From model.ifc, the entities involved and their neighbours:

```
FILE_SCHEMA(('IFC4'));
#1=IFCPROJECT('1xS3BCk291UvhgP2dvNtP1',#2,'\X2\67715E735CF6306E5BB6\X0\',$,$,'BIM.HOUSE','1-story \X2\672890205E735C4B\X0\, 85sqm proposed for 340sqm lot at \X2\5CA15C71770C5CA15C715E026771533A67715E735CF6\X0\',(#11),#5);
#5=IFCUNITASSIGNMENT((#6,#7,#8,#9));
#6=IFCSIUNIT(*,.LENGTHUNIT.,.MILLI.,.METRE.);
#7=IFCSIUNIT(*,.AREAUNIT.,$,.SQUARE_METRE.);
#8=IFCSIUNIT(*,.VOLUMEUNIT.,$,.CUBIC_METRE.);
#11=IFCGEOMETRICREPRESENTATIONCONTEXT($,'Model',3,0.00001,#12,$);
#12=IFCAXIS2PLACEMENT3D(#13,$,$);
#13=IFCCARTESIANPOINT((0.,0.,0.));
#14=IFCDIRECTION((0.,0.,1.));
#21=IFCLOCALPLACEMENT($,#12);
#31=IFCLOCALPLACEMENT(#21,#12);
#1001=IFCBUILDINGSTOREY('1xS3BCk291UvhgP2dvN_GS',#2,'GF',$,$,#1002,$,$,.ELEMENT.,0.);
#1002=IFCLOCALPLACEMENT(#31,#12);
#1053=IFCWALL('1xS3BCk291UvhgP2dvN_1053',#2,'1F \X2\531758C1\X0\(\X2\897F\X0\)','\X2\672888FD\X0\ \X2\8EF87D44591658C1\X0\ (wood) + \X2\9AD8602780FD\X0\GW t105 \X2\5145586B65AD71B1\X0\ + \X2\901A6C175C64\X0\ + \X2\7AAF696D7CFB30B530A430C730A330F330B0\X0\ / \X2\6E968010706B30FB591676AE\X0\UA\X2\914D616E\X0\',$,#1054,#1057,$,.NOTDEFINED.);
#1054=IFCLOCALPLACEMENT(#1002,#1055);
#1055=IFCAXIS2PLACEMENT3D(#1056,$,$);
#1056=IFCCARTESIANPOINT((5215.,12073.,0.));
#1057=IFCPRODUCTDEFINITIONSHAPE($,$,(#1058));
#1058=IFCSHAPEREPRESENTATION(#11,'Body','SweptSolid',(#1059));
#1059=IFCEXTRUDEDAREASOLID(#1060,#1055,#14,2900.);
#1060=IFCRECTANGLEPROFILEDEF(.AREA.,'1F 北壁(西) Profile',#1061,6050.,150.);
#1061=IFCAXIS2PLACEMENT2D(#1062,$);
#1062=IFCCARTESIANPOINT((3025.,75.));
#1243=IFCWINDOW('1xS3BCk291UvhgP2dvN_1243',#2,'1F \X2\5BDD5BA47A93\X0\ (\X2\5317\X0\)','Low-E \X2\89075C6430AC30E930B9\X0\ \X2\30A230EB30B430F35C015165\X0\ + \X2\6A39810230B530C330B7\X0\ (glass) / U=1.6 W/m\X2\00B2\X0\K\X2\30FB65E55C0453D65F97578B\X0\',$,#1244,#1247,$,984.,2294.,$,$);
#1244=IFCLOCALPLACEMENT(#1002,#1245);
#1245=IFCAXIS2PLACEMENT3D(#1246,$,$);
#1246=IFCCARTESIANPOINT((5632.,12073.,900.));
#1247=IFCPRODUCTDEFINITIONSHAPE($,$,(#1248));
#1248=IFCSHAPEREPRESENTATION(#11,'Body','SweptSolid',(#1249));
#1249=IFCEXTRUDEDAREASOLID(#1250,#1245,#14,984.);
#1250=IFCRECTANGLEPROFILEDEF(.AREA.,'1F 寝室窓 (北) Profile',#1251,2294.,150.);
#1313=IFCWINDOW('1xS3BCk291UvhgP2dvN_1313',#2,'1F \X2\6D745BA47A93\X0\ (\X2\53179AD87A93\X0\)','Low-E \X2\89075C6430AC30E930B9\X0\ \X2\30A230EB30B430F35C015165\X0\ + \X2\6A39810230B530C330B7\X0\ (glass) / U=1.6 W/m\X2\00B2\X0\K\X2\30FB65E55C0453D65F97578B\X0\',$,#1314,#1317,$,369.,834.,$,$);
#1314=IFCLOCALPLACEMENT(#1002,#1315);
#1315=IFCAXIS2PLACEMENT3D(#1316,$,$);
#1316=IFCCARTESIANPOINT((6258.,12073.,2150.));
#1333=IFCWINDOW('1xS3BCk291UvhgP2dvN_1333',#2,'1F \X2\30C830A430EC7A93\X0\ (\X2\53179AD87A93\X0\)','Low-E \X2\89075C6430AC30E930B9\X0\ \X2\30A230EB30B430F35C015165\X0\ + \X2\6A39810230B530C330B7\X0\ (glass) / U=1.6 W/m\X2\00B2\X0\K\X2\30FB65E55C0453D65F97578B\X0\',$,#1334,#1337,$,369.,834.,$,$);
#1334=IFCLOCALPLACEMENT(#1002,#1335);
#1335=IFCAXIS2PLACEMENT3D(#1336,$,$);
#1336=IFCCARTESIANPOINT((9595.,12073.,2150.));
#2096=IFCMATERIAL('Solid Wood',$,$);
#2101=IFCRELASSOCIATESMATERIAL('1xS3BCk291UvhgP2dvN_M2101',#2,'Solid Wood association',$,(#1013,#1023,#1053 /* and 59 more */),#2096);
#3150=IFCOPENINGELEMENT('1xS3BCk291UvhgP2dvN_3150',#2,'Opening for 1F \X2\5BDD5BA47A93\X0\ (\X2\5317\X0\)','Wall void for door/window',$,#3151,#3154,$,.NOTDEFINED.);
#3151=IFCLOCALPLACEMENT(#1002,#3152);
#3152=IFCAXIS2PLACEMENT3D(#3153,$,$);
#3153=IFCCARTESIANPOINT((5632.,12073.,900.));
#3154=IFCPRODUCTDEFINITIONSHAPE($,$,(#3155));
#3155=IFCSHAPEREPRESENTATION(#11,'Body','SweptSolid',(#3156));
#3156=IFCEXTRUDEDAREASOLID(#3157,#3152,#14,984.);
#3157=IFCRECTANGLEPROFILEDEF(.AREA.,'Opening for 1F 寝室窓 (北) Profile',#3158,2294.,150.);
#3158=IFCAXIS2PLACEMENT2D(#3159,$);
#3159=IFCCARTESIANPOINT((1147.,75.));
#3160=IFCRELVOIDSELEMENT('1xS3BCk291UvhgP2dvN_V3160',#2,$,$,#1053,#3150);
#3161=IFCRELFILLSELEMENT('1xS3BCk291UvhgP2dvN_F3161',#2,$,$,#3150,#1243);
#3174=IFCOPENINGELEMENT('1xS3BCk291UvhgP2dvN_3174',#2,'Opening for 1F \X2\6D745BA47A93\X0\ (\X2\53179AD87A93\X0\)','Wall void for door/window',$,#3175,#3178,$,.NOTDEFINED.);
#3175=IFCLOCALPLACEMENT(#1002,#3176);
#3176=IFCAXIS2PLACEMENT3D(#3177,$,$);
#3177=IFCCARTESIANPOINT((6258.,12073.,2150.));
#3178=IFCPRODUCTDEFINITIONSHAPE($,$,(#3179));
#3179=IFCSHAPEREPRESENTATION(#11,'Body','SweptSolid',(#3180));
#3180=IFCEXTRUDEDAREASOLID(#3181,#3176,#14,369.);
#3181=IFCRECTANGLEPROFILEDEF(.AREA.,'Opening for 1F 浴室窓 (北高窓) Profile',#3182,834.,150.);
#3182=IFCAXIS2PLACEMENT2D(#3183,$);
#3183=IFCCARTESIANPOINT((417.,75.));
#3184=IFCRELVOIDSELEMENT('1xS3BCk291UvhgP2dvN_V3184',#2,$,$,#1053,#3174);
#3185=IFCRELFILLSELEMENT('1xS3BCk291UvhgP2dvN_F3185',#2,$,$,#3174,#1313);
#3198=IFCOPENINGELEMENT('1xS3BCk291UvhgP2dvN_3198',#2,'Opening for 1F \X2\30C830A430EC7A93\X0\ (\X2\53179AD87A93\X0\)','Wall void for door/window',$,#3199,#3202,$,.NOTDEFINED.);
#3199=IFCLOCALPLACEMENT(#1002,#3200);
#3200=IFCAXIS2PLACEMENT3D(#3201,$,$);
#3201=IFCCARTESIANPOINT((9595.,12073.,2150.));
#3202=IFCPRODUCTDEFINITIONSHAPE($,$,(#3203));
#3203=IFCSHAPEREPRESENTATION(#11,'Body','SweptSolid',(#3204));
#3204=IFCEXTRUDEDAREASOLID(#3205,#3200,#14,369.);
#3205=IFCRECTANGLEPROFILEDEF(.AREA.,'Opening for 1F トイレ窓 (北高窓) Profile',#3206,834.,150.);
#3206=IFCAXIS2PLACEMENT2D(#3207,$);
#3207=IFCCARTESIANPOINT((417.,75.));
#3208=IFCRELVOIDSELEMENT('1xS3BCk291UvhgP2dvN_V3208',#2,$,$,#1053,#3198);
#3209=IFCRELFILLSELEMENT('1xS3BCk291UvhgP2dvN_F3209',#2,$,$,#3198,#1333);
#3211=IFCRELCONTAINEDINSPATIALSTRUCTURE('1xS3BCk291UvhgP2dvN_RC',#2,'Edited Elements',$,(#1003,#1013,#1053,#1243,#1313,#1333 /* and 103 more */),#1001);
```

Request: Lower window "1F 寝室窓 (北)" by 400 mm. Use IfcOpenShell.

```python
import numpy as np
import ifcopenshell
import ifcopenshell.api.geometry
import ifcopenshell.util.placement
import ifcopenshell.util.unit

model = ifcopenshell.open("model.ifc")
unit_scale = ifcopenshell.util.unit.calculate_unit_scale(model)

window = model.by_id(1243)
opening = window.FillsVoids[0].RelatingOpeningElement
dz = -400.0

shift = np.array([0.0, 0.0, dz])
# The window is not placed relative to its opening, so move both.
for product in (opening, window):
    matrix = ifcopenshell.util.placement.get_local_placement(product.ObjectPlacement)
    matrix[:3, 3] += shift
    ifcopenshell.api.geometry.edit_object_placement(model, product=product, matrix=matrix, is_si=False)

print(f"moved by {dz * unit_scale:+.3f} m")

model.write("model_edited.ifc")
```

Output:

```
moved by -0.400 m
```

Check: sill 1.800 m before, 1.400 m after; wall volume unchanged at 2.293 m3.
